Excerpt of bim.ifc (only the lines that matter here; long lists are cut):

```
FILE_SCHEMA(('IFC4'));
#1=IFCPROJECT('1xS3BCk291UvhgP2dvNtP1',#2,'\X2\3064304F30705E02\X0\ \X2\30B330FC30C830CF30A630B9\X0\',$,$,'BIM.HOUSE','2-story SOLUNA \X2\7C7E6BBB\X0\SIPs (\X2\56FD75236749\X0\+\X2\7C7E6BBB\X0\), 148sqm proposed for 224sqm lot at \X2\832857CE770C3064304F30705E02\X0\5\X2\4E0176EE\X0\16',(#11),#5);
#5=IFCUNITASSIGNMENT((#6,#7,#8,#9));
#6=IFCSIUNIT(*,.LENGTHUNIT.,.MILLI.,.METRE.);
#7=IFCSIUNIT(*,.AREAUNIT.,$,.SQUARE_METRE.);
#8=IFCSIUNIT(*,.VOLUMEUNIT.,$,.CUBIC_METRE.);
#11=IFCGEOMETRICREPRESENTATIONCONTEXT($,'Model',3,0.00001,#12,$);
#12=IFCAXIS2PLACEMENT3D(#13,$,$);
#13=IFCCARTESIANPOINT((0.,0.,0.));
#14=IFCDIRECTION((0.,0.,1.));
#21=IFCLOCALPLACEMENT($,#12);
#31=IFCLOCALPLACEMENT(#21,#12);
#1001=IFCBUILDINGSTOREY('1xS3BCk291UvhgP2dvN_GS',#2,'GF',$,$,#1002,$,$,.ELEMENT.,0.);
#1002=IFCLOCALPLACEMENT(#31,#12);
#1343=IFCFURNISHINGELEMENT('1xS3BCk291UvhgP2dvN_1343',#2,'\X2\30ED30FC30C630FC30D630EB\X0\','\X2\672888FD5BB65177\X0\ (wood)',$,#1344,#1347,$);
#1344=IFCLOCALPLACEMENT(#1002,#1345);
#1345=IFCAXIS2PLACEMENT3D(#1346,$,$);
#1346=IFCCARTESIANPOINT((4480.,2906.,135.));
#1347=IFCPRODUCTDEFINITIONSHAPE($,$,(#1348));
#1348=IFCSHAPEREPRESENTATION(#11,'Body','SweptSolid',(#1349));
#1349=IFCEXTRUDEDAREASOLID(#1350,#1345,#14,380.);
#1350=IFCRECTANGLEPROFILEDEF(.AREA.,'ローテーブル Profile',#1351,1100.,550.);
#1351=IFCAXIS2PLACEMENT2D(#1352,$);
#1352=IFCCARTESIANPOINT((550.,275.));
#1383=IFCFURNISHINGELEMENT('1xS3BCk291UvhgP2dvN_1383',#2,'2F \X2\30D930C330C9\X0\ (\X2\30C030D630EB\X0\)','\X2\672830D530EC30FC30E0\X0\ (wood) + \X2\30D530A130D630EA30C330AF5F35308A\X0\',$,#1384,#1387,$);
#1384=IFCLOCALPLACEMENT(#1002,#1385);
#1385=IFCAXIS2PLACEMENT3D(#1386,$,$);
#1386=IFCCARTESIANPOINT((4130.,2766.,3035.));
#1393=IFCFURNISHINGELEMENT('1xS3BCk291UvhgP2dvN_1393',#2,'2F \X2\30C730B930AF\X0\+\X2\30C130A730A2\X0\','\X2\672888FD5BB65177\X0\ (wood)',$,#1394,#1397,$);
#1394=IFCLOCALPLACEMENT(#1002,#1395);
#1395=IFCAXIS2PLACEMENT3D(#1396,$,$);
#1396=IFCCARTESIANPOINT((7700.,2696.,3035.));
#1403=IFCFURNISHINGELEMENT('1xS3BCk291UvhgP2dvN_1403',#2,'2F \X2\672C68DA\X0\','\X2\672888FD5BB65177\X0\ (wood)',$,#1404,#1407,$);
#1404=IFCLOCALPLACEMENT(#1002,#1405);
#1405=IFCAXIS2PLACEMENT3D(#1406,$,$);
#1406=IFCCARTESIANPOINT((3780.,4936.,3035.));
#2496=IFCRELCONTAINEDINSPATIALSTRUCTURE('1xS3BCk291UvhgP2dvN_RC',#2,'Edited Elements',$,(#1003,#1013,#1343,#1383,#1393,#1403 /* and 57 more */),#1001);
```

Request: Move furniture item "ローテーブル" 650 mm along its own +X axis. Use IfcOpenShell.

```python
import ifcopenshell
import ifcopenshell.api.geometry
import ifcopenshell.util.placement
import ifcopenshell.util.unit

model = ifcopenshell.open("bim.ifc")
unit_scale = ifcopenshell.util.unit.calculate_unit_scale(model)

item = model.by_id(1343)
matrix = ifcopenshell.util.placement.get_local_placement(item.ObjectPlacement)
matrix[:3, 3] += matrix[:3, 0] * 0.65 / unit_scale
ifcopenshell.api.geometry.edit_object_placement(model, product=item, matrix=matrix, is_si=False)

print(ifcopenshell.util.placement.get_local_placement(item.ObjectPlacement).round(3) + 0.0)

model.write("bim_rev.ifc")
```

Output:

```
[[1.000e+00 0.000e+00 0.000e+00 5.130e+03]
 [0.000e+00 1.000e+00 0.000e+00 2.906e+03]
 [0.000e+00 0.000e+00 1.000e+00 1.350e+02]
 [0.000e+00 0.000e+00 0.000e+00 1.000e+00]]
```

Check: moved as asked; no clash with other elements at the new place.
